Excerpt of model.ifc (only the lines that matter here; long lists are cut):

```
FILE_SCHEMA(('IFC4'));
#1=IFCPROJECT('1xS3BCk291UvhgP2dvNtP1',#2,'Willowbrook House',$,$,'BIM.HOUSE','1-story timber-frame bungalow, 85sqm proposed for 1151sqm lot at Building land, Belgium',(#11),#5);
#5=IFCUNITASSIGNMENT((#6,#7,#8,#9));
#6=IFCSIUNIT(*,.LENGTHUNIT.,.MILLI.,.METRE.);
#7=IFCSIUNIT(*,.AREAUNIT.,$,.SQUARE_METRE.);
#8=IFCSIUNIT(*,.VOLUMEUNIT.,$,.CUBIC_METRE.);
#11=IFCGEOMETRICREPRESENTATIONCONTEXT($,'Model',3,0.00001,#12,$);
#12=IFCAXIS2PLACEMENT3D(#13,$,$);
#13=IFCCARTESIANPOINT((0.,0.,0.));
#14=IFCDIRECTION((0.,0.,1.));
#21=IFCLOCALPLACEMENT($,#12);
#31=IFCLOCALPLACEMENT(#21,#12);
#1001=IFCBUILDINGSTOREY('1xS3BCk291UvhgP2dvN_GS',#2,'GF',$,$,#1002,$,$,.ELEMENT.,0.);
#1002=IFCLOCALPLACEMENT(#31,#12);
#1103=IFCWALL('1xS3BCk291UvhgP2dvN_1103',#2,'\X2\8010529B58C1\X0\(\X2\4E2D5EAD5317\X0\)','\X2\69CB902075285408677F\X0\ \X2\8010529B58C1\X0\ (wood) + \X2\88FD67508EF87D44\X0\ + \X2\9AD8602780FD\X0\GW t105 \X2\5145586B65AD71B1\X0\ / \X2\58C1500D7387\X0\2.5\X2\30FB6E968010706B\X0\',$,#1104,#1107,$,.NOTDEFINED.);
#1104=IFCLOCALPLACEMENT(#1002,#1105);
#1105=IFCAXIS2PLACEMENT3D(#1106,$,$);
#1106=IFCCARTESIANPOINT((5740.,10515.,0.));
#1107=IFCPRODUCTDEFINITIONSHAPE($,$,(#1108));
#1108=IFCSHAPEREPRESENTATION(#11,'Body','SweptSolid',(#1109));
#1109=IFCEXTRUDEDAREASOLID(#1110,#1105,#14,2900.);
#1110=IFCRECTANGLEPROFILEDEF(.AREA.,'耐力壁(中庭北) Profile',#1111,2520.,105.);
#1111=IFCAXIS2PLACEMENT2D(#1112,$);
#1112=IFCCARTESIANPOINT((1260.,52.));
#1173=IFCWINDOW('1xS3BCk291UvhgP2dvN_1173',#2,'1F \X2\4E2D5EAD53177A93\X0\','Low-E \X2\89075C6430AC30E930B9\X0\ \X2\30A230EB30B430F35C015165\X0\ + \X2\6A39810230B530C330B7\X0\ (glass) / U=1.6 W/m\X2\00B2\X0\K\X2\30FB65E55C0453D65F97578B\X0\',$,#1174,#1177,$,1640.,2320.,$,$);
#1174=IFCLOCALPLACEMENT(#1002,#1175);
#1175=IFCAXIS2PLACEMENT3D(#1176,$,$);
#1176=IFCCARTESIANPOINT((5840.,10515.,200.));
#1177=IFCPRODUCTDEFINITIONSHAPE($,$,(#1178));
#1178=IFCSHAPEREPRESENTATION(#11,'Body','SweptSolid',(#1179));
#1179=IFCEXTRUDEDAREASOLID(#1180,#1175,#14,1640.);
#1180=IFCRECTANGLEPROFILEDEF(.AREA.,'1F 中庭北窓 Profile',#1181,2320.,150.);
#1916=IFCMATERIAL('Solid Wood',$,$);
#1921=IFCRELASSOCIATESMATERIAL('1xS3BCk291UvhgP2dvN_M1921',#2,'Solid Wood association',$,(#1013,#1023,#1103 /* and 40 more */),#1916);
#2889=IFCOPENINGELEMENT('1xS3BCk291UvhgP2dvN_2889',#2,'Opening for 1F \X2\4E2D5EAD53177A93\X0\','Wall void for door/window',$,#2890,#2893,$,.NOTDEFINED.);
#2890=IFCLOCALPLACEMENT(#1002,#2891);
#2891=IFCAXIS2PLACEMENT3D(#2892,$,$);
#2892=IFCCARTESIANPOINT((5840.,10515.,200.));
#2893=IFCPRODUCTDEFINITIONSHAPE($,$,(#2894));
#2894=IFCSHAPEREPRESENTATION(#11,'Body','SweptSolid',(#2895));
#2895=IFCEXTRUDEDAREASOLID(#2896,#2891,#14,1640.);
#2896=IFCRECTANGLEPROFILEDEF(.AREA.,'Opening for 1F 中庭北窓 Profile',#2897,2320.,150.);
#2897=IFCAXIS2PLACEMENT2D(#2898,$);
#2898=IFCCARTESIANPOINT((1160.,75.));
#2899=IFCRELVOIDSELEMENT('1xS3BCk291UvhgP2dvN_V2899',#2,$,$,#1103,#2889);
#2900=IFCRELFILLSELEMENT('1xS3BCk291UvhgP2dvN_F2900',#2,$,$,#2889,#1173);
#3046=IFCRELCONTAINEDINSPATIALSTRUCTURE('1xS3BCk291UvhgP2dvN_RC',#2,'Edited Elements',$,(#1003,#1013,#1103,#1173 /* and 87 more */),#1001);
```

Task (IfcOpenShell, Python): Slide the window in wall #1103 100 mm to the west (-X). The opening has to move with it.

```python
import ifcopenshell
import ifcopenshell.api.geometry
import ifcopenshell.util.placement
import ifcopenshell.util.unit

model = ifcopenshell.open("model.ifc")
unit_scale = ifcopenshell.util.unit.calculate_unit_scale(model)

window = model.by_guid("1xS3BCk291UvhgP2dvN_1173")
opening = window.FillsVoids[0].RelatingOpeningElement
wall = opening.VoidsElements[0].RelatingBuildingElement

wall_matrix = ifcopenshell.util.placement.get_local_placement(wall.ObjectPlacement)
shift = wall_matrix[:3, 0] * -0.1 / unit_scale
before = ifcopenshell.util.placement.get_local_placement(window.ObjectPlacement)[:3, 3].copy()

# The window is not placed relative to its opening, so move both.
for product in (opening, window):
    matrix = ifcopenshell.util.placement.get_local_placement(product.ObjectPlacement)
    matrix[:3, 3] += shift
    ifcopenshell.api.geometry.edit_object_placement(model, product=product, matrix=matrix, is_si=False)

after = ifcopenshell.util.placement.get_local_placement(window.ObjectPlacement)[:3, 3]
print("window moved by", (after - before).round(3) + 0.0)

model.write("model-out.ifc")
```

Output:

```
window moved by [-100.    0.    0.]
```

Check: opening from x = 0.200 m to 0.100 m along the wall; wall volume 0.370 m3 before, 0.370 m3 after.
